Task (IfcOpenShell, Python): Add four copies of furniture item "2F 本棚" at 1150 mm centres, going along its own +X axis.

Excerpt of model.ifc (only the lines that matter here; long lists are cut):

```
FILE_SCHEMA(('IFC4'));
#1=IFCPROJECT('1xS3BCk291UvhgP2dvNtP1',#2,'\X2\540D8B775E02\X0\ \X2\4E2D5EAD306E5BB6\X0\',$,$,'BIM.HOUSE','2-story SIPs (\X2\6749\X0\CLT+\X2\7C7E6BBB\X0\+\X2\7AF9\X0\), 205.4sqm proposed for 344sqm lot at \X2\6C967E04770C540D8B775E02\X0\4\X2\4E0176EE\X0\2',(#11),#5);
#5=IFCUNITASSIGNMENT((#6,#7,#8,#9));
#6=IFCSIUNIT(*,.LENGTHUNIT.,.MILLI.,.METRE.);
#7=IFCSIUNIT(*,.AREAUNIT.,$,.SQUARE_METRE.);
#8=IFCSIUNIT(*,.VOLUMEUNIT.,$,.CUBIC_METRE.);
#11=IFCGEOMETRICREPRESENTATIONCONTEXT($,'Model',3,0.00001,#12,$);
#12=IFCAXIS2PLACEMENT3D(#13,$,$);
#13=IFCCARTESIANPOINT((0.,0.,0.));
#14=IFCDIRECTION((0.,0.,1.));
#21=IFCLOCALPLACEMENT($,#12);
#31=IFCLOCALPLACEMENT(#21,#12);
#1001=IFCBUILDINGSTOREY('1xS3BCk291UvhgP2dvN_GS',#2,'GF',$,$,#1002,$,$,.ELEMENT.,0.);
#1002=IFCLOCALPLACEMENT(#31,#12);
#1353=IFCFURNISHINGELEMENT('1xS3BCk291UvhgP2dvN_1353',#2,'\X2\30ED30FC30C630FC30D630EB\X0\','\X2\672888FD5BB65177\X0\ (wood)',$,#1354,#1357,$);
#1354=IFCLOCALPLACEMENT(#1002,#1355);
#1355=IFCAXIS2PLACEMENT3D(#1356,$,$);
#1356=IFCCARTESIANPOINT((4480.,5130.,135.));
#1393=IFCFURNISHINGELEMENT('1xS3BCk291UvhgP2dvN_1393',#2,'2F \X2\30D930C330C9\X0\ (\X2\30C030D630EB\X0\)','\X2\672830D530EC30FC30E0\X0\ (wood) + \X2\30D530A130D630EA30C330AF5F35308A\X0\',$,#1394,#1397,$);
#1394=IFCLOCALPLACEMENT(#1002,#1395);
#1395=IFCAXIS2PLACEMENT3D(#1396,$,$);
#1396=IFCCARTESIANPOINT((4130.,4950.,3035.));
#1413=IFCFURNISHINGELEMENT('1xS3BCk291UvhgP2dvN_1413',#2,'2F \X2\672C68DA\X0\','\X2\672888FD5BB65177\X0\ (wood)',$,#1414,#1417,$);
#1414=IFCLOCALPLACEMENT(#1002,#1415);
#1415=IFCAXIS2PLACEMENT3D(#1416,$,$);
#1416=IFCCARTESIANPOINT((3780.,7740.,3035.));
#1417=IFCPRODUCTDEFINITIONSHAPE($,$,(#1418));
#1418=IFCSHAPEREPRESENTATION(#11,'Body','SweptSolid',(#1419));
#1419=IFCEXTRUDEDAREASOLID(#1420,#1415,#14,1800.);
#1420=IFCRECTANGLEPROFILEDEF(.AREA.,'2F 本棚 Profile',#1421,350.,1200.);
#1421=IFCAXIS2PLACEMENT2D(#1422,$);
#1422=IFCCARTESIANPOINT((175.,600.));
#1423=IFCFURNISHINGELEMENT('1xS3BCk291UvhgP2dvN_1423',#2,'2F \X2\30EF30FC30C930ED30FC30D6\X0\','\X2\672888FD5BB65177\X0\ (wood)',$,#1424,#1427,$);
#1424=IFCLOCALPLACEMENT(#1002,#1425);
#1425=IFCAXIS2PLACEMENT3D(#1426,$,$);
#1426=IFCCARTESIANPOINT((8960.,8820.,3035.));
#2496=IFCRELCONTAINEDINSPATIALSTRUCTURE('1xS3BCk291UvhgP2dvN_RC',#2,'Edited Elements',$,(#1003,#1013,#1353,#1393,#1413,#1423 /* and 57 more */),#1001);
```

```python
import ifcopenshell
import ifcopenshell.api.geometry
import ifcopenshell.api.root
import ifcopenshell.util.element
import ifcopenshell.util.placement
import ifcopenshell.util.unit

model = ifcopenshell.open("model.ifc")
unit_scale = ifcopenshell.util.unit.calculate_unit_scale(model)


def reuse_history(source, copy):
    """copy_class also copies each property set's owner history, people and application; keep the originals."""
    for rel in copy.IsDefinedBy:
        if rel.is_a("IfcRelDefinesByProperties") and (history := rel.RelatingPropertyDefinition.OwnerHistory):
            rel.RelatingPropertyDefinition.OwnerHistory = source.OwnerHistory
            ifcopenshell.util.element.remove_deep2(model, history)


source = model.by_guid("1xS3BCk291UvhgP2dvN_1413")
base = ifcopenshell.util.placement.get_local_placement(source.ObjectPlacement)
step = base[:3, 0] * 1.15 / unit_scale

for i in range(1, 5):
    copy = ifcopenshell.api.root.copy_class(model, product=source)
    copy.Representation = ifcopenshell.util.element.copy_deep(
        model, source.Representation, exclude=["IfcGeometricRepresentationContext", "IfcRepresentationMap"]
    )
    reuse_history(source, copy)
    matrix = base.copy()
    matrix[:3, 3] += i * step
    print("added at", matrix[:3, 3].round(3) + 0.0)
    ifcopenshell.api.geometry.edit_object_placement(model, product=copy, matrix=matrix, is_si=False)

model.write("model_edited.ifc")
```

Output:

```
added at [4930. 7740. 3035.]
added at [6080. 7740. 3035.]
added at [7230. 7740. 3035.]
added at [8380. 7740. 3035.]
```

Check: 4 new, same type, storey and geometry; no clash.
